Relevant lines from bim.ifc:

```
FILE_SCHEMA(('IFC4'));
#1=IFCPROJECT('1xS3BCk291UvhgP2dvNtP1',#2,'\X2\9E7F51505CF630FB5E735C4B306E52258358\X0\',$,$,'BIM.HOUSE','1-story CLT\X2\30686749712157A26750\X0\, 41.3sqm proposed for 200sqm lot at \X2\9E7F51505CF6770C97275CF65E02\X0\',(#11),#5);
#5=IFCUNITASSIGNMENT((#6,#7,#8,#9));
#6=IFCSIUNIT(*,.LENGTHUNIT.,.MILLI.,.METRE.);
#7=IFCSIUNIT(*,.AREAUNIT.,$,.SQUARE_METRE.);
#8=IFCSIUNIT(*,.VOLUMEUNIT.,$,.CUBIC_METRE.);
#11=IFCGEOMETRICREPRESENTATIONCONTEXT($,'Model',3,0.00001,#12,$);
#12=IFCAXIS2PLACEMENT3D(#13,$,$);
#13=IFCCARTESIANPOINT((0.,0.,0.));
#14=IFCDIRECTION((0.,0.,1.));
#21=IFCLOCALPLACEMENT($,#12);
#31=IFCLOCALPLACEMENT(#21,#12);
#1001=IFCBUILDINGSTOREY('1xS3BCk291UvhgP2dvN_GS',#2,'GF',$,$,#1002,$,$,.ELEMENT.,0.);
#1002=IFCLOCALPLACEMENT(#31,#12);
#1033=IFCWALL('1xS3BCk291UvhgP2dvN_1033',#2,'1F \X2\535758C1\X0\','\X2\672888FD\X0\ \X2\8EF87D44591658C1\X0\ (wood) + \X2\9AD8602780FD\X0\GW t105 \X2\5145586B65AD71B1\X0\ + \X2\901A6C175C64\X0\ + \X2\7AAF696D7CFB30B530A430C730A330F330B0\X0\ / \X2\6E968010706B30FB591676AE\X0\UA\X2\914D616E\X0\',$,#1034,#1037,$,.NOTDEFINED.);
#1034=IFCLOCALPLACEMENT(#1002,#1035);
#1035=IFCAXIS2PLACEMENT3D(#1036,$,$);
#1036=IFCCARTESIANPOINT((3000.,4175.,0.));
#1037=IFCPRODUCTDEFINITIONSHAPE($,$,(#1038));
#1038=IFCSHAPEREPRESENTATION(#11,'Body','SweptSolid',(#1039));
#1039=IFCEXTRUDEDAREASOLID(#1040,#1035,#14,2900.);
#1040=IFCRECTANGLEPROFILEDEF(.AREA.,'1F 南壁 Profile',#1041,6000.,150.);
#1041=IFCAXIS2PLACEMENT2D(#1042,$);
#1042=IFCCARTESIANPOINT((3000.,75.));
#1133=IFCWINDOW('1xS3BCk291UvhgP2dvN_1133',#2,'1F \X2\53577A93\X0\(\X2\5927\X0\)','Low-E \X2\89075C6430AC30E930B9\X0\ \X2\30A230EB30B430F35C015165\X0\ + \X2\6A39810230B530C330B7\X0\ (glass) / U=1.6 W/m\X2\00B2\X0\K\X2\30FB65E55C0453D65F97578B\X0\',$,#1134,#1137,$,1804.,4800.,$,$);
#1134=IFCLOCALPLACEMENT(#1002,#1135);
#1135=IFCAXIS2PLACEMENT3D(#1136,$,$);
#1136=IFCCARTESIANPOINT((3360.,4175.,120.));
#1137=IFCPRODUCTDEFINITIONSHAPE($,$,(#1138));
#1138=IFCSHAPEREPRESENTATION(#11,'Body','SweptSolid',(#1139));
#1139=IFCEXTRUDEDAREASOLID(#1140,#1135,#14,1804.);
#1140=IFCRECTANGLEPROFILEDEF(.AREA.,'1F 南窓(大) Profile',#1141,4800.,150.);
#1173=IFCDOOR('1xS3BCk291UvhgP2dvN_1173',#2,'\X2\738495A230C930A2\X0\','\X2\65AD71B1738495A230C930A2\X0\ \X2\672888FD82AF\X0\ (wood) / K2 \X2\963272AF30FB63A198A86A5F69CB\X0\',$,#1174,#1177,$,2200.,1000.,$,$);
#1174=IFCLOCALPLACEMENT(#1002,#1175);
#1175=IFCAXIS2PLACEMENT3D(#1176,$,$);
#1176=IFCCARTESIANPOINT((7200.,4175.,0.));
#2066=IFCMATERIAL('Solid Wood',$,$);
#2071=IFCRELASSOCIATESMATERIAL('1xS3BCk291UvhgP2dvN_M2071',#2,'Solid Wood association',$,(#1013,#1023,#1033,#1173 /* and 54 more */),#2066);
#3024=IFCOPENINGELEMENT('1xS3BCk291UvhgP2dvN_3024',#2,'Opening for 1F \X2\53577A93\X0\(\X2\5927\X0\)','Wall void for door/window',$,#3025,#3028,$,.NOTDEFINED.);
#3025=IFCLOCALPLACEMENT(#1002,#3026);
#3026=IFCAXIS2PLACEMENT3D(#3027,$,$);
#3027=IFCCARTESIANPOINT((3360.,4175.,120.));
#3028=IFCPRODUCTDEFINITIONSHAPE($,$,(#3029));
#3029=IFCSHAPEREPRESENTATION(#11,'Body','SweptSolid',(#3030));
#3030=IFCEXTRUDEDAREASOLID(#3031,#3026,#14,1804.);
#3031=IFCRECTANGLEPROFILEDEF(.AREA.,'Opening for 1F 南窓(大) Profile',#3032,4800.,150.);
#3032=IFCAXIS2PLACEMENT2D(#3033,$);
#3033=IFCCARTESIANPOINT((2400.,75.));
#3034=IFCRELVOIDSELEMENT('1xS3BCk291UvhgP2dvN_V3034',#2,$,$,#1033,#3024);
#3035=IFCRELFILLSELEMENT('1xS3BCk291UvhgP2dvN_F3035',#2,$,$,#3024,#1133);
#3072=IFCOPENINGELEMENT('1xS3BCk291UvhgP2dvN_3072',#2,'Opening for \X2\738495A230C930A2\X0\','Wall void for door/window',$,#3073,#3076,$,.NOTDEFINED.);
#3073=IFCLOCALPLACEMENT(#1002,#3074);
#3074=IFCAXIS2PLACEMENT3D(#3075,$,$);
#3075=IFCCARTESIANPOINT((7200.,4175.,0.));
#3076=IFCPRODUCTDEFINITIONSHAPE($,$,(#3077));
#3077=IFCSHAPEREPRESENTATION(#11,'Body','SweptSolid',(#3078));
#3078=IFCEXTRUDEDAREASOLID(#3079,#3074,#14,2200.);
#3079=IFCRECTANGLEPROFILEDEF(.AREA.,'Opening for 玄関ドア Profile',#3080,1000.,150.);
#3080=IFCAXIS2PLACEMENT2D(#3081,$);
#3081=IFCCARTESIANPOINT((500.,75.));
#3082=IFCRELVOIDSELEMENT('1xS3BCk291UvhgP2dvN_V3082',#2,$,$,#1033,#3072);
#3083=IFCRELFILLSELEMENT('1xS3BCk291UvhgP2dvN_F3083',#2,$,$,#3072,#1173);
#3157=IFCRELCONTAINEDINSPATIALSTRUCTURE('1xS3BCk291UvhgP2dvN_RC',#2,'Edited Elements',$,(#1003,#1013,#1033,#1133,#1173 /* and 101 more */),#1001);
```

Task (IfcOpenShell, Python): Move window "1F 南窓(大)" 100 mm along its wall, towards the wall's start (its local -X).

```python
import ifcopenshell
import ifcopenshell.api.geometry
import ifcopenshell.util.placement
import ifcopenshell.util.unit

model = ifcopenshell.open("bim.ifc")
unit_scale = ifcopenshell.util.unit.calculate_unit_scale(model)

window = model.by_guid("1xS3BCk291UvhgP2dvN_1133")
opening = window.FillsVoids[0].RelatingOpeningElement
wall = opening.VoidsElements[0].RelatingBuildingElement

wall_matrix = ifcopenshell.util.placement.get_local_placement(wall.ObjectPlacement)
shift = wall_matrix[:3, 0] * -0.1 / unit_scale
before = ifcopenshell.util.placement.get_local_placement(window.ObjectPlacement)[:3, 3].copy()

# The window is not placed relative to its opening, so move both.
for product in (opening, window):
    matrix = ifcopenshell.util.placement.get_local_placement(product.ObjectPlacement)
    matrix[:3, 3] += shift
    ifcopenshell.api.geometry.edit_object_placement(model, product=product, matrix=matrix, is_si=False)

after = ifcopenshell.util.placement.get_local_placement(window.ObjectPlacement)[:3, 3]
print("window moved by", (after - before).round(3) + 0.0)

model.write("bim-out.ifc")
```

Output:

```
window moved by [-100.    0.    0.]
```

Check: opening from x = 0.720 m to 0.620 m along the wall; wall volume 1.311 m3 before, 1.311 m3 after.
